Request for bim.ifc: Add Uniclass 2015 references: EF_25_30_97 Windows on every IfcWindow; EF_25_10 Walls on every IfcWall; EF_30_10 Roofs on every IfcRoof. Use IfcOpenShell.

First a look at what the model holds.

```python
import ifcopenshell

model = ifcopenshell.open("bim.ifc")
print(model.schema)
print("classifications:", [c.Name for c in model.by_type("IfcClassification")])
for ifc_class in ("IfcDoor", "IfcRoof", "IfcStair", "IfcWall", "IfcWindow"):
    print(ifc_class, len(model.by_type(ifc_class)))
```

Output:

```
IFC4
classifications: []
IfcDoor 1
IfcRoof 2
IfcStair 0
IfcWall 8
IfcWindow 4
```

```python
import ifcopenshell
import ifcopenshell.api.classification

model = ifcopenshell.open("bim.ifc")

system = ifcopenshell.api.classification.add_classification(model, classification="Uniclass 2015")

codes = {
    "IfcWindow": ("EF_25_30_97", "Windows"),
    "IfcWall": ("EF_25_10", "Walls"),
    "IfcRoof": ("EF_30_10", "Roofs"),
}
for ifc_class, (code, name) in codes.items():
    products = model.by_type(ifc_class)
    ifcopenshell.api.classification.add_reference(
        model, products=products, classification=system, identification=code, name=name
    )
    print(code, len(products))

model.write("bim_updated.ifc")
```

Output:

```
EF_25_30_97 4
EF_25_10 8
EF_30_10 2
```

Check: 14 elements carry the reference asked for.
